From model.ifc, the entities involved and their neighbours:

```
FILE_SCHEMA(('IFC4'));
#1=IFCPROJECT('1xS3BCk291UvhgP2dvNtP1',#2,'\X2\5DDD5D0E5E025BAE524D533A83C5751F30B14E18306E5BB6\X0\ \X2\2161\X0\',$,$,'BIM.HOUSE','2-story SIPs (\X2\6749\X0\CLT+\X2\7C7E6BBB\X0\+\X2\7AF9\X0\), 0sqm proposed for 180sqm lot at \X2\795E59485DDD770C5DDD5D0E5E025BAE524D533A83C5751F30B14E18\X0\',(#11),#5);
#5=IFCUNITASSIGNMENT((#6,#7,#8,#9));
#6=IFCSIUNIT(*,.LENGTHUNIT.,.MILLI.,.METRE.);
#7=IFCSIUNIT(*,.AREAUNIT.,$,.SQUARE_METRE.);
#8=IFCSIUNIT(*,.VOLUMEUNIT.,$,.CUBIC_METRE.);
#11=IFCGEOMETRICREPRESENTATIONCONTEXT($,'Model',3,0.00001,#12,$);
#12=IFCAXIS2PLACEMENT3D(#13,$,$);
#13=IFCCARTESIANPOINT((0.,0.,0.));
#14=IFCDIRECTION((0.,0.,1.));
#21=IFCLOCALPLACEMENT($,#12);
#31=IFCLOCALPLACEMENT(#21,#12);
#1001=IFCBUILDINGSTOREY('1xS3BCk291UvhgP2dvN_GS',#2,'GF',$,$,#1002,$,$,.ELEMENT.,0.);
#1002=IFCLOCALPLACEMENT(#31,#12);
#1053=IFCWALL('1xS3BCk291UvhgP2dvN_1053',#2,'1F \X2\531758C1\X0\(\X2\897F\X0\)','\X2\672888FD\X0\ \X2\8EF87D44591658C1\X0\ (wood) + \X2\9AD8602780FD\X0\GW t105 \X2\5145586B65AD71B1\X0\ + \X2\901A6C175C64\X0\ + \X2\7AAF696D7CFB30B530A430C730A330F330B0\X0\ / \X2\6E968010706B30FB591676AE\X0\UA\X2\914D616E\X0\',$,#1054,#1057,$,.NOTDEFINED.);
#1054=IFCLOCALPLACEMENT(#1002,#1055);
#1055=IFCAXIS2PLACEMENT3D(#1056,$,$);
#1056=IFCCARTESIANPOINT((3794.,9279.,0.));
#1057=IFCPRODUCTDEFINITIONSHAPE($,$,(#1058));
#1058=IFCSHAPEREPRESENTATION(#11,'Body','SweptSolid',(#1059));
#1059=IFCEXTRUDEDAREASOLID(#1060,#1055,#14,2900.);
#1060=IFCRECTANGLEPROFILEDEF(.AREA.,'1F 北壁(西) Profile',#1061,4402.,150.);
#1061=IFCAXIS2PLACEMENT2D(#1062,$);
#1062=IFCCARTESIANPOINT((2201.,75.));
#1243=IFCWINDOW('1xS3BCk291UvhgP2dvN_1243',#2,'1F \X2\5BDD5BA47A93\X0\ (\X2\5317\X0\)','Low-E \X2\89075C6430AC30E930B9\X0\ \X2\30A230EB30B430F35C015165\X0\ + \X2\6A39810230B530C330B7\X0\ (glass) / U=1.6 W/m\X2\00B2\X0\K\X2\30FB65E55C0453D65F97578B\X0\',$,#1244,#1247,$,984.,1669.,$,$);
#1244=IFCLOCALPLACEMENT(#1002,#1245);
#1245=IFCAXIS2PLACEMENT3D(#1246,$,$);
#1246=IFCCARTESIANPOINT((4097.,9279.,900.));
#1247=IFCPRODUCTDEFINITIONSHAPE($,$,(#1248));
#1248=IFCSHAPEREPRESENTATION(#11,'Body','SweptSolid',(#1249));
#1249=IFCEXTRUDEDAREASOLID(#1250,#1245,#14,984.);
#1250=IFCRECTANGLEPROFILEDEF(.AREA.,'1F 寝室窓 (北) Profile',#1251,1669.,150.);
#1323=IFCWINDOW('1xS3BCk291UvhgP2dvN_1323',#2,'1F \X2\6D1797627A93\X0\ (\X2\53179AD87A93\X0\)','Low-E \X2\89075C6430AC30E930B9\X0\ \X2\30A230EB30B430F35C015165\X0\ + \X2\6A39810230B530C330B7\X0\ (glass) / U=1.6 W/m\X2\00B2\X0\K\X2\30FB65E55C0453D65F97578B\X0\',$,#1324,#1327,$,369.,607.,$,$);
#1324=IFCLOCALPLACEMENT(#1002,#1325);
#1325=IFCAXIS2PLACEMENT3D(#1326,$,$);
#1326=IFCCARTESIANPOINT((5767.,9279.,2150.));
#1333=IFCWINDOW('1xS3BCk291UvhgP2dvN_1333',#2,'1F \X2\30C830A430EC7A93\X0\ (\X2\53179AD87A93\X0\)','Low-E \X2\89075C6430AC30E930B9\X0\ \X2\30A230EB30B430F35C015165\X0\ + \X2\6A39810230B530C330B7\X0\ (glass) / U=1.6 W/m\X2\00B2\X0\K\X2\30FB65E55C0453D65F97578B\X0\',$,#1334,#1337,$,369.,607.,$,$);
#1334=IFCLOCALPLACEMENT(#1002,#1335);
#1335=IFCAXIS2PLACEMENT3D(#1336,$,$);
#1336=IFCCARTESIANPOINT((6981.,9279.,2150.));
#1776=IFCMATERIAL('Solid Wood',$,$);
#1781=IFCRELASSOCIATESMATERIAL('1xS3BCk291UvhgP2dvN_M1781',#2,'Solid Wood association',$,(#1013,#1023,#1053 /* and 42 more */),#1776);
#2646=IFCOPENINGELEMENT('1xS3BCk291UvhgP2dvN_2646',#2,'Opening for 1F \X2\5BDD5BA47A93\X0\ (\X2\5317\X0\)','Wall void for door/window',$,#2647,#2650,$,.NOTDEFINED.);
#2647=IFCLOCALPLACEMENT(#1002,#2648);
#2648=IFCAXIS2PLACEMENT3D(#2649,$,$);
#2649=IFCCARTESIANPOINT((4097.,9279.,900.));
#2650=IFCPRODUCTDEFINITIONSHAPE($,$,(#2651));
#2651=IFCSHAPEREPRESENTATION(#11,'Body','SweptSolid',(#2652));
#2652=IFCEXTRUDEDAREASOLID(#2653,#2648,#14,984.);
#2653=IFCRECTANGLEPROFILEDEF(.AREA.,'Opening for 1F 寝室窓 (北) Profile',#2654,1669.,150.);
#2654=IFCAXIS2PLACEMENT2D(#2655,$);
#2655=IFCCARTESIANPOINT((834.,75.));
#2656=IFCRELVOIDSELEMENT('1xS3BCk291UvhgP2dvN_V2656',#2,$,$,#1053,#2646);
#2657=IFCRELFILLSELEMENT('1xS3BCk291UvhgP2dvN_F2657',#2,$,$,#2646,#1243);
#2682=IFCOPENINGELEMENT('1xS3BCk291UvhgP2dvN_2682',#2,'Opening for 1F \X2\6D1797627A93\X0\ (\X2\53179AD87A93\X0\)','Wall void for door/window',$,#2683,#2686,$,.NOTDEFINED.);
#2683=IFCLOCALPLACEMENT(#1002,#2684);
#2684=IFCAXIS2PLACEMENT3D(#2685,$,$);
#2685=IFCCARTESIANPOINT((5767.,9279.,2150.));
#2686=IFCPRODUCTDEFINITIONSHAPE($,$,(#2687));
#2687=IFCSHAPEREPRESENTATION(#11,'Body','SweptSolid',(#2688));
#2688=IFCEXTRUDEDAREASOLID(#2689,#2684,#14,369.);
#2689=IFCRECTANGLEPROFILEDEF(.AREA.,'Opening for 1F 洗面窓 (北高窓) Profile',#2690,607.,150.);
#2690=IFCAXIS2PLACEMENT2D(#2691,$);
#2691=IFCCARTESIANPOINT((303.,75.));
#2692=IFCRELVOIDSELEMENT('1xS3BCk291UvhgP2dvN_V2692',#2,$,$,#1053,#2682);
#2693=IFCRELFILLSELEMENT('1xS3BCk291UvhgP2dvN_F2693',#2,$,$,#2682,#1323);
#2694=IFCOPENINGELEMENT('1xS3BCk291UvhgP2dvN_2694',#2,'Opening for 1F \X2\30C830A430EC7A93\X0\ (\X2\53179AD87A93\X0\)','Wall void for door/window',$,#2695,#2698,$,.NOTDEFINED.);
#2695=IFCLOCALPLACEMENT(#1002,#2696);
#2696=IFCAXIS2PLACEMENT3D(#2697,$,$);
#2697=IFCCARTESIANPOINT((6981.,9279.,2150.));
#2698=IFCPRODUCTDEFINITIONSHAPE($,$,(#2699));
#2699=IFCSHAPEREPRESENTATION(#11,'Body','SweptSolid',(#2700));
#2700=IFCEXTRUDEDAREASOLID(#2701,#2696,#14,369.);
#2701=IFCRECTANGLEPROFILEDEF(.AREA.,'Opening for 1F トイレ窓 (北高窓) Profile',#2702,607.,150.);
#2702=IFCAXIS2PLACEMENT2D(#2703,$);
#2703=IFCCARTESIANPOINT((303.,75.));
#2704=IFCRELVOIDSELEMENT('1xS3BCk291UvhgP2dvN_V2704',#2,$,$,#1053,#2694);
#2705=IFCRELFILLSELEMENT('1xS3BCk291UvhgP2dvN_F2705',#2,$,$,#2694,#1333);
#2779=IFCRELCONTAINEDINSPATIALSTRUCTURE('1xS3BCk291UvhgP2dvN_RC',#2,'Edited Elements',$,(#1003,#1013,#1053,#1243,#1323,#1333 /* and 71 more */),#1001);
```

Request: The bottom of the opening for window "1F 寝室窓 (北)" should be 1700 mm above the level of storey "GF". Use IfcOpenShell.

```python
import numpy as np
import ifcopenshell
import ifcopenshell.api.geometry
import ifcopenshell.geom
import ifcopenshell.util.element
import ifcopenshell.util.placement
import ifcopenshell.util.shape
import ifcopenshell.util.unit

model = ifcopenshell.open("model.ifc")
unit_scale = ifcopenshell.util.unit.calculate_unit_scale(model)

window = model.by_guid("1xS3BCk291UvhgP2dvN_1243")
opening = window.FillsVoids[0].RelatingOpeningElement
storey = ifcopenshell.util.element.get_container(window, ifc_class="IfcBuildingStorey")
level = ifcopenshell.util.placement.get_local_placement(storey.ObjectPlacement)[2, 3]

# The opening's origin need not be at the sill, so measure its lowest point.
shape = ifcopenshell.geom.create_shape(ifcopenshell.geom.settings(), opening)
bottom = ifcopenshell.util.shape.get_shape_bottom_elevation(shape, shape.geometry) / unit_scale
dz = level + 1.7 / unit_scale - bottom

shift = np.array([0.0, 0.0, dz])
# The window is not placed relative to its opening, so move both.
for product in (opening, window):
    matrix = ifcopenshell.util.placement.get_local_placement(product.ObjectPlacement)
    matrix[:3, 3] += shift
    ifcopenshell.api.geometry.edit_object_placement(model, product=product, matrix=matrix, is_si=False)

print(f"moved by {dz * unit_scale:+.3f} m")

model.write("model-out.ifc")
```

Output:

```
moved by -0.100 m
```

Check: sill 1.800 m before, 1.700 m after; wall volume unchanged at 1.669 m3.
